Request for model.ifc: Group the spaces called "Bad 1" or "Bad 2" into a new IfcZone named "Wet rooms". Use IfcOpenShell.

First a look at what the model holds.

```python
import ifcopenshell

model = ifcopenshell.open("model.ifc")
print(model.schema)
seen = {}
for space in model.by_type("IfcSpace"):
    seen[space.LongName] = seen.get(space.LongName, 0) + 1
for name, count in sorted(seen.items(), key=str):
    print(count, "x", name)
print("zones:", [z.Name for z in model.by_type("IfcZone")][:20])
```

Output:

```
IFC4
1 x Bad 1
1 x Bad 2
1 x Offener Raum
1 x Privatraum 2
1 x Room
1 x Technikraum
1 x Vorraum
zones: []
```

```python
import ifcopenshell
import ifcopenshell.api.group
import ifcopenshell.api.root

model = ifcopenshell.open("model.ifc")

names = {"Bad 1", "Bad 2"}
spaces = [s for s in model.by_type("IfcSpace") if s.LongName in names]

zone = ifcopenshell.api.root.create_entity(model, ifc_class="IfcZone", name="Wet rooms")
ifcopenshell.api.group.assign_group(model, products=spaces, group=zone)
print(len(spaces), "spaces in", zone.Name)

model.write("model_rev.ifc")
```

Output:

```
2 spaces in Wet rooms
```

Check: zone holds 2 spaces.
